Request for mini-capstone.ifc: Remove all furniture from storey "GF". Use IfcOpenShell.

First a look at what the model holds.

```python
import ifcopenshell
import ifcopenshell.util.element

model = ifcopenshell.open("mini-capstone.ifc")
print(model.schema)
storey = next(s for s in model.by_type("IfcBuildingStorey") if s.Name == "GF")
furniture = [e for e in ifcopenshell.util.element.get_decomposition(storey) if e.is_a("IfcFurnishingElement")]
seen = {}
for e in furniture:
    element_type = ifcopenshell.util.element.get_type(e)
    name = element_type.Name if element_type not in (None, e) else None
    seen[name] = seen.get(name, 0) + 1
for name, count in sorted(seen.items(), key=str):
    print(count, "x", name)
```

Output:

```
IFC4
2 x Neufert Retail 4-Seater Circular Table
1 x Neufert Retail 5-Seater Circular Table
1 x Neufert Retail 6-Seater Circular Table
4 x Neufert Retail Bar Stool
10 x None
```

```python
import ifcopenshell
import ifcopenshell.api.root
import ifcopenshell.util.element

model = ifcopenshell.open("mini-capstone.ifc")

storey = next(s for s in model.by_type("IfcBuildingStorey") if s.Name == "GF")
furniture = [e for e in ifcopenshell.util.element.get_decomposition(storey) if e.is_a("IfcFurnishingElement")]

for e in furniture:
    ifcopenshell.api.root.remove_product(model, product=e)
print(len(furniture), "removed")

model.write("mini-capstone_edited.ifc")
```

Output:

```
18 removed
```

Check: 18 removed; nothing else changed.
